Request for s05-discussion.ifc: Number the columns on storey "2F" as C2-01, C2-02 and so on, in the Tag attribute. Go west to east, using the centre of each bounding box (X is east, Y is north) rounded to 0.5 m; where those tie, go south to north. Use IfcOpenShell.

First a look at what the model holds.

```python
import ifcopenshell
import ifcopenshell.util.element
import ifcopenshell.util.placement

model = ifcopenshell.open("s05-discussion.ifc")
print(model.schema)
storey = next(s for s in model.by_type("IfcBuildingStorey") if s.Name == "2F")
columns = [e for e in ifcopenshell.util.element.get_decomposition(storey) if e.is_a("IfcColumn")]
for e in sorted(columns, key=lambda e: e.id()):
    origin = ifcopenshell.util.placement.get_local_placement(e.ObjectPlacement)[:3, 3]
    print(e.id(), e.Tag, e.Name, origin.round(2) + 0.0, sep=" | ")
```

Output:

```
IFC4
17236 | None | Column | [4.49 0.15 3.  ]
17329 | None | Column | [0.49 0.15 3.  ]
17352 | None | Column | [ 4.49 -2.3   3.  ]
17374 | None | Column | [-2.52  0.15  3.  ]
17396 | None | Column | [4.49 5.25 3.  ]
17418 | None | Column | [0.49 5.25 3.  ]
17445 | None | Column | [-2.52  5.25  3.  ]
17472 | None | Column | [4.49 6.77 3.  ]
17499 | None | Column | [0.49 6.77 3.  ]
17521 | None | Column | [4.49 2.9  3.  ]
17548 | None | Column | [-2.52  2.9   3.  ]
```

```python
import ifcopenshell
import ifcopenshell.geom
import ifcopenshell.util.element
import ifcopenshell.util.shape

model = ifcopenshell.open("s05-discussion.ifc")
settings = ifcopenshell.geom.settings()
settings.set("use-world-coords", True)


def centre(element):
    shape = ifcopenshell.geom.create_shape(settings, element)
    return ifcopenshell.util.shape.get_bbox_centroid(shape.geometry)


storey = next(s for s in model.by_type("IfcBuildingStorey") if s.Name == "2F")
columns = [e for e in ifcopenshell.util.element.get_decomposition(storey) if e.is_a("IfcColumn")]

# Insertion points can sit at a corner or the storey origin, so sort by the geometry (in metres).
centres = {e: centre(e) for e in columns}
columns.sort(key=lambda e: (round(centres[e][0] / 0.5), centres[e][1]))

for i, e in enumerate(columns, start=1):
    number = f"C2-{i:02d}"
    e.Tag = number
    print(e.id(), number)

model.write("s05-discussion_edited.ifc")
```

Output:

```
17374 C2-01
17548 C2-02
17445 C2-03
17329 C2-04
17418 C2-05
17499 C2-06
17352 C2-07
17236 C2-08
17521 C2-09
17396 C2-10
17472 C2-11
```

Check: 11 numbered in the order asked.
